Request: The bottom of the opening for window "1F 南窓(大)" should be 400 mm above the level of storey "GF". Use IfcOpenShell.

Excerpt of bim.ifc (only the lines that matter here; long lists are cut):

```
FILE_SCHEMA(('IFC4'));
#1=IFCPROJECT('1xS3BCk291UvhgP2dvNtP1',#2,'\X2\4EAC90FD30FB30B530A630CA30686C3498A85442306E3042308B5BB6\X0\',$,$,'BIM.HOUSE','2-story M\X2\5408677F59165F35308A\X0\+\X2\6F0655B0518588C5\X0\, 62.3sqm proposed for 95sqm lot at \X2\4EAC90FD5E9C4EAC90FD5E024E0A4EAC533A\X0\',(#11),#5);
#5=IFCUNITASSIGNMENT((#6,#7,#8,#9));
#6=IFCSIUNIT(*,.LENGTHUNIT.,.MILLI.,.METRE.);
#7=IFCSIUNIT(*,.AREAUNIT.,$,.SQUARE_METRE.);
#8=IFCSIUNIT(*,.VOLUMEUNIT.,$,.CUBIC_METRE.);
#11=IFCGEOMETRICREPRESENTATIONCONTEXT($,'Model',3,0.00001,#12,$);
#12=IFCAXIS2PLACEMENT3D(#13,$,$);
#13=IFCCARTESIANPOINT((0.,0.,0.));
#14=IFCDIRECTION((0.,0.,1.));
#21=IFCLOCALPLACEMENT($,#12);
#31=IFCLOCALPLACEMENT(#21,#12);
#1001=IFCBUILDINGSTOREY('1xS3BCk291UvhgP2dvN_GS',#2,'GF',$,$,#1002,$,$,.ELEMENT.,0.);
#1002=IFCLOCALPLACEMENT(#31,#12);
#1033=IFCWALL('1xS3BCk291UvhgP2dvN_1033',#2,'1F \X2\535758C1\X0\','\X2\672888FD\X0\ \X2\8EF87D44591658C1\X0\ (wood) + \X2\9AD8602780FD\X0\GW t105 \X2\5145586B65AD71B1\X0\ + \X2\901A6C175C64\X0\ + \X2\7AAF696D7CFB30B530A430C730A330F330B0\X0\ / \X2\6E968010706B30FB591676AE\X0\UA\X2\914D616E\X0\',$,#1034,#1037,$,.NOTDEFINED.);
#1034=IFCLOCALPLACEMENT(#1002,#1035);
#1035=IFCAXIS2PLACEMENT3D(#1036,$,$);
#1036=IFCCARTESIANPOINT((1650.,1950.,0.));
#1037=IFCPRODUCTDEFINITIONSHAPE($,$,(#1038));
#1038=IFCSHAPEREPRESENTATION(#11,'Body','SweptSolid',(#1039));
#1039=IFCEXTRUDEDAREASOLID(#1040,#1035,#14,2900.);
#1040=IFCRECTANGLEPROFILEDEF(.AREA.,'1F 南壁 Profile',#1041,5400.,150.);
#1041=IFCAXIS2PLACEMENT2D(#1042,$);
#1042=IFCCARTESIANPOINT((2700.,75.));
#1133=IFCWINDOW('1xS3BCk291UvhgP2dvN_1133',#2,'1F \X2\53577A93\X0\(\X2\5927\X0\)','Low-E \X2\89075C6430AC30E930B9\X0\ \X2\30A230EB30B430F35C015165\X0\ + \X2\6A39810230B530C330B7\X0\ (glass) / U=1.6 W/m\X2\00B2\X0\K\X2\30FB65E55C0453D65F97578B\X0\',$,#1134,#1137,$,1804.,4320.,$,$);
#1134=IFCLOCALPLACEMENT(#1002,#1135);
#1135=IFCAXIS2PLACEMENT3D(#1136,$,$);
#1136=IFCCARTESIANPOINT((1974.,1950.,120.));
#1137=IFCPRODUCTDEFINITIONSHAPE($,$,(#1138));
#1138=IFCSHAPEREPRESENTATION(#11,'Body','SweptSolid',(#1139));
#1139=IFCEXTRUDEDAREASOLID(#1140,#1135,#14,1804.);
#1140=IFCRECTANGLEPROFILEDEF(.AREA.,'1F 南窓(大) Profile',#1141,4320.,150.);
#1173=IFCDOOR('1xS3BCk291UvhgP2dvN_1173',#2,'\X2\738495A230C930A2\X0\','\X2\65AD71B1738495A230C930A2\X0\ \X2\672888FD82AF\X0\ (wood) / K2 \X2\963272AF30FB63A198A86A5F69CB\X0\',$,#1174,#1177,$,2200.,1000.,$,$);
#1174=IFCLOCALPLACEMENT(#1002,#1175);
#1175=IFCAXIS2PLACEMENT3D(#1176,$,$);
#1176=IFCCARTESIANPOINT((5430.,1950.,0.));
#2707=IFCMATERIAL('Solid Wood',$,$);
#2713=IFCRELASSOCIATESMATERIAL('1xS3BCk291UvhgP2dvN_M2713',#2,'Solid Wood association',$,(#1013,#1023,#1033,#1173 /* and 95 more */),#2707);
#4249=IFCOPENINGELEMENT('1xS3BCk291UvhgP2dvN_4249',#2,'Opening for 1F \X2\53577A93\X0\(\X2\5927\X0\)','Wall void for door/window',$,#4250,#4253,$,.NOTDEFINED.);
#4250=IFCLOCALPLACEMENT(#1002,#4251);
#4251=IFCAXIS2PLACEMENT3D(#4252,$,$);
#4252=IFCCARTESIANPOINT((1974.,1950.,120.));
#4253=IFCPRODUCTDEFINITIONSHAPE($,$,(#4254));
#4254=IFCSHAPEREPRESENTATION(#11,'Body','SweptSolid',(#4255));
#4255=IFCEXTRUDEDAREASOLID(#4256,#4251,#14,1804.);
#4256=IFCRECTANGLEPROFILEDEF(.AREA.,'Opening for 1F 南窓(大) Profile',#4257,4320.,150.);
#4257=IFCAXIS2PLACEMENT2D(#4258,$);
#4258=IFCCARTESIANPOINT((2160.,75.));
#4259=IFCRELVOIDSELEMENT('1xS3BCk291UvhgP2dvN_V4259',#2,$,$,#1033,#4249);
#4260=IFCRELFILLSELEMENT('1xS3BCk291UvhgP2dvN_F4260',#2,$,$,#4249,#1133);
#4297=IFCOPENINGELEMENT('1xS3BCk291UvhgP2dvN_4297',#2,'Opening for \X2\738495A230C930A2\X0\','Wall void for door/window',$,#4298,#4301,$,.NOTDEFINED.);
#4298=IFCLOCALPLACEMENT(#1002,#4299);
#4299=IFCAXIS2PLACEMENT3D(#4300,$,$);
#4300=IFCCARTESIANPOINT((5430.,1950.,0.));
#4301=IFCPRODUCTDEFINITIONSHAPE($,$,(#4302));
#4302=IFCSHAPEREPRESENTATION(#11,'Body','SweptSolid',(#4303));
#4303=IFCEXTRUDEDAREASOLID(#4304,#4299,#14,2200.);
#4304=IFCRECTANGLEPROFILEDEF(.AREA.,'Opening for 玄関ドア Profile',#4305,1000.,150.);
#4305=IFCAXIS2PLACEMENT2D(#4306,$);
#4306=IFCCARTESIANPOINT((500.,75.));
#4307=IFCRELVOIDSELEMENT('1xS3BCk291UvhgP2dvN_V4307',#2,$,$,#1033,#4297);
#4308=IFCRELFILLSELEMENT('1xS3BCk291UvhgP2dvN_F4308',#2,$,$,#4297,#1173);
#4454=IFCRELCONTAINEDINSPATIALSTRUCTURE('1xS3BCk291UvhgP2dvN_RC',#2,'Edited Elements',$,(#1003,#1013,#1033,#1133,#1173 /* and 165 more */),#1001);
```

```python
import numpy as np
import ifcopenshell
import ifcopenshell.api.geometry
import ifcopenshell.geom
import ifcopenshell.util.element
import ifcopenshell.util.placement
import ifcopenshell.util.shape
import ifcopenshell.util.unit

model = ifcopenshell.open("bim.ifc")
unit_scale = ifcopenshell.util.unit.calculate_unit_scale(model)

window = model.by_guid("1xS3BCk291UvhgP2dvN_1133")
opening = window.FillsVoids[0].RelatingOpeningElement
storey = ifcopenshell.util.element.get_container(window, ifc_class="IfcBuildingStorey")
level = ifcopenshell.util.placement.get_local_placement(storey.ObjectPlacement)[2, 3]

# The opening's origin need not be at the sill, so measure its lowest point.
shape = ifcopenshell.geom.create_shape(ifcopenshell.geom.settings(), opening)
bottom = ifcopenshell.util.shape.get_shape_bottom_elevation(shape, shape.geometry) / unit_scale
dz = level + 0.4 / unit_scale - bottom

shift = np.array([0.0, 0.0, dz])
# The window is not placed relative to its opening, so move both.
for product in (opening, window):
    matrix = ifcopenshell.util.placement.get_local_placement(product.ObjectPlacement)
    matrix[:3, 3] += shift
    ifcopenshell.api.geometry.edit_object_placement(model, product=product, matrix=matrix, is_si=False)

print(f"moved by {dz * unit_scale:+.3f} m")

model.write("bim_edited.ifc")
```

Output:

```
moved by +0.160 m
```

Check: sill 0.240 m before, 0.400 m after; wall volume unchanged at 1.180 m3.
